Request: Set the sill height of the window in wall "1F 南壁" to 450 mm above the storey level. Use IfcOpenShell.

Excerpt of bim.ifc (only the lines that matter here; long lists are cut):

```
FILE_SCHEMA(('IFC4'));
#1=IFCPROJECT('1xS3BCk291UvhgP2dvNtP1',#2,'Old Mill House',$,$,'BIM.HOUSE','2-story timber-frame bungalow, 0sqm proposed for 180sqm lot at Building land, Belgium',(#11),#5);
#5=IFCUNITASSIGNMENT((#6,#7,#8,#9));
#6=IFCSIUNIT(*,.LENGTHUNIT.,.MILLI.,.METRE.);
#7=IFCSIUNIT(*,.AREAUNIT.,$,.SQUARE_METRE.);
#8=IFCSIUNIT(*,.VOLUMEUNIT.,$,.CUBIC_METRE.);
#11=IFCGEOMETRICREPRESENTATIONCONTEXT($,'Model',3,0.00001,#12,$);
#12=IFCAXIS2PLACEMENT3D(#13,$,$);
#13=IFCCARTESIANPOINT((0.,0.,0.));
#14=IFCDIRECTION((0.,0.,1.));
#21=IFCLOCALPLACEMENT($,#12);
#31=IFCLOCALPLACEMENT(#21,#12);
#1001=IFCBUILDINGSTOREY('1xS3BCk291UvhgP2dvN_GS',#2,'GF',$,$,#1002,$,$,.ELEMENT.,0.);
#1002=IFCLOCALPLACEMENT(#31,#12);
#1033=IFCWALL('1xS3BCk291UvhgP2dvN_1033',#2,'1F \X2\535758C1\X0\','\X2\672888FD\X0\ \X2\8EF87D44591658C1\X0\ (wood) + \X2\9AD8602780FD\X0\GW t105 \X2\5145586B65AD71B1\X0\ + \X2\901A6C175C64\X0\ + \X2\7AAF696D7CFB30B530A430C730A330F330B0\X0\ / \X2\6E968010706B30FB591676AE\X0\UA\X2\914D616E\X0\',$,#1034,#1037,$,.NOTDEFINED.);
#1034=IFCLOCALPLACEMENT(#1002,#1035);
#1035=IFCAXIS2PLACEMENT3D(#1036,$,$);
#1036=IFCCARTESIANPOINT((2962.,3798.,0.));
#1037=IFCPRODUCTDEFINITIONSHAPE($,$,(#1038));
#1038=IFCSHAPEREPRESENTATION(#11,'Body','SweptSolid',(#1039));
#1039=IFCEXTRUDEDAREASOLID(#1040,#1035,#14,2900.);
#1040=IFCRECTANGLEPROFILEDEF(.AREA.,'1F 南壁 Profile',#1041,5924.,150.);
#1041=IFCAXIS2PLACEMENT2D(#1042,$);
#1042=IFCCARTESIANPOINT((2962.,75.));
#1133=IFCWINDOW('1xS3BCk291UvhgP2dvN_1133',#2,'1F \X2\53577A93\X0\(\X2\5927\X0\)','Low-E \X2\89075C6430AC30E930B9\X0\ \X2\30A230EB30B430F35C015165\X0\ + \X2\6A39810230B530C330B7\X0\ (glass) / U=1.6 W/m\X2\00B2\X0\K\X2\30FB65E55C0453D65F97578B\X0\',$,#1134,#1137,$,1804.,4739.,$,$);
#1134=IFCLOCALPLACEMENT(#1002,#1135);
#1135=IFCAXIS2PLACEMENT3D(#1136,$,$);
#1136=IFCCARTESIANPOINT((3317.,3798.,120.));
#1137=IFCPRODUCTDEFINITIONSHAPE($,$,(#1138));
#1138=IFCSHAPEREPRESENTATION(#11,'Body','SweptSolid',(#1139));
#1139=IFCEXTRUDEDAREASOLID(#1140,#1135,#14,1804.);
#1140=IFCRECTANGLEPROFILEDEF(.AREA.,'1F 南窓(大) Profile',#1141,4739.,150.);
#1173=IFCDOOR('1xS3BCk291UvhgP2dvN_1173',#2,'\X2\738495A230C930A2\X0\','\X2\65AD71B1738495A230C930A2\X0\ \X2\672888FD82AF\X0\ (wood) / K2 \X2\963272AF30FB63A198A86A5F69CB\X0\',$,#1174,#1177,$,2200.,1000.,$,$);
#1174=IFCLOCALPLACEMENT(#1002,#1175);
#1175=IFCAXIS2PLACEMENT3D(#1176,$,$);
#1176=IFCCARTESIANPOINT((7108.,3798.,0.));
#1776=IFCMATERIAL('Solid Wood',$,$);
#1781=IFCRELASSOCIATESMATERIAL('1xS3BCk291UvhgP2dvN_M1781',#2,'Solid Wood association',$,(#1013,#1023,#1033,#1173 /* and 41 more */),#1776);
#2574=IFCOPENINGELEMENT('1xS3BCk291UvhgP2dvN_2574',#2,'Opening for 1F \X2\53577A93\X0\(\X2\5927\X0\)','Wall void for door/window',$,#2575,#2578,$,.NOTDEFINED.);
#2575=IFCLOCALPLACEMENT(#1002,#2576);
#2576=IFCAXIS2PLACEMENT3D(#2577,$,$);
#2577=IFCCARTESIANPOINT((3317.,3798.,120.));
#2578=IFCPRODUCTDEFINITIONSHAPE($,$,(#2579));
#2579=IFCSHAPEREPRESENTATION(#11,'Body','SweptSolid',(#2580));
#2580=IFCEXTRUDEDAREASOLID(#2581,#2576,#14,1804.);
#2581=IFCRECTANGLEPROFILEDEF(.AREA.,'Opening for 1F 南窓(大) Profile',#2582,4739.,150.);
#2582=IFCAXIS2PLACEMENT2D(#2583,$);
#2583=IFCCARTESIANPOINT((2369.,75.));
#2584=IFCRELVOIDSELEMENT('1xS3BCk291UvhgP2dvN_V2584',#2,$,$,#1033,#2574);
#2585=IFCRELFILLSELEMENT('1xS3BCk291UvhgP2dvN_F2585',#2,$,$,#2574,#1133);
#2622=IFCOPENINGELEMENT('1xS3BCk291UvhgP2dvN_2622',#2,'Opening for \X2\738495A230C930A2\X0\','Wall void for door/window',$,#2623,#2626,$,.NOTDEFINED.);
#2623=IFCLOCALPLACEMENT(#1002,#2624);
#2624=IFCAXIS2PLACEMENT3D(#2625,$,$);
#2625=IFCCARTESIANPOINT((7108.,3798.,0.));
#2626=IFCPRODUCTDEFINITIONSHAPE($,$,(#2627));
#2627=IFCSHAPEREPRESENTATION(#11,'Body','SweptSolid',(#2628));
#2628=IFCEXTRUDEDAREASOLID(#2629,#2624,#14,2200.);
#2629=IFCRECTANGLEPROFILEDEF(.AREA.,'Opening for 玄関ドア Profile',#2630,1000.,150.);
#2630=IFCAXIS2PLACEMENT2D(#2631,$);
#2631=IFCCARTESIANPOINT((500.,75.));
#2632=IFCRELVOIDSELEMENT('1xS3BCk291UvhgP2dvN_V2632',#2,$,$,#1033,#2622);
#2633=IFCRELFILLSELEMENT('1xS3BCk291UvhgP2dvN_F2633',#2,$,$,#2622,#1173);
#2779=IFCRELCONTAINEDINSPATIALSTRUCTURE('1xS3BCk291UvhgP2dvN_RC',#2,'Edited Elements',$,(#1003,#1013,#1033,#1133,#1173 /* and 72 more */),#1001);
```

```python
import numpy as np
import ifcopenshell
import ifcopenshell.api.geometry
import ifcopenshell.geom
import ifcopenshell.util.element
import ifcopenshell.util.placement
import ifcopenshell.util.shape
import ifcopenshell.util.unit

model = ifcopenshell.open("bim.ifc")
unit_scale = ifcopenshell.util.unit.calculate_unit_scale(model)

window = model.by_guid("1xS3BCk291UvhgP2dvN_1133")
opening = window.FillsVoids[0].RelatingOpeningElement
storey = ifcopenshell.util.element.get_container(window, ifc_class="IfcBuildingStorey")
level = ifcopenshell.util.placement.get_local_placement(storey.ObjectPlacement)[2, 3]

# The opening's origin need not be at the sill, so measure its lowest point.
shape = ifcopenshell.geom.create_shape(ifcopenshell.geom.settings(), opening)
bottom = ifcopenshell.util.shape.get_shape_bottom_elevation(shape, shape.geometry) / unit_scale
dz = level + 0.45 / unit_scale - bottom

shift = np.array([0.0, 0.0, dz])
# The window is not placed relative to its opening, so move both.
for product in (opening, window):
    matrix = ifcopenshell.util.placement.get_local_placement(product.ObjectPlacement)
    matrix[:3, 3] += shift
    ifcopenshell.api.geometry.edit_object_placement(model, product=product, matrix=matrix, is_si=False)

print(f"moved by {dz * unit_scale:+.3f} m")

model.write("bim_updated.ifc")
```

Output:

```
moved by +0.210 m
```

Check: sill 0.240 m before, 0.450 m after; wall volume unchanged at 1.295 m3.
